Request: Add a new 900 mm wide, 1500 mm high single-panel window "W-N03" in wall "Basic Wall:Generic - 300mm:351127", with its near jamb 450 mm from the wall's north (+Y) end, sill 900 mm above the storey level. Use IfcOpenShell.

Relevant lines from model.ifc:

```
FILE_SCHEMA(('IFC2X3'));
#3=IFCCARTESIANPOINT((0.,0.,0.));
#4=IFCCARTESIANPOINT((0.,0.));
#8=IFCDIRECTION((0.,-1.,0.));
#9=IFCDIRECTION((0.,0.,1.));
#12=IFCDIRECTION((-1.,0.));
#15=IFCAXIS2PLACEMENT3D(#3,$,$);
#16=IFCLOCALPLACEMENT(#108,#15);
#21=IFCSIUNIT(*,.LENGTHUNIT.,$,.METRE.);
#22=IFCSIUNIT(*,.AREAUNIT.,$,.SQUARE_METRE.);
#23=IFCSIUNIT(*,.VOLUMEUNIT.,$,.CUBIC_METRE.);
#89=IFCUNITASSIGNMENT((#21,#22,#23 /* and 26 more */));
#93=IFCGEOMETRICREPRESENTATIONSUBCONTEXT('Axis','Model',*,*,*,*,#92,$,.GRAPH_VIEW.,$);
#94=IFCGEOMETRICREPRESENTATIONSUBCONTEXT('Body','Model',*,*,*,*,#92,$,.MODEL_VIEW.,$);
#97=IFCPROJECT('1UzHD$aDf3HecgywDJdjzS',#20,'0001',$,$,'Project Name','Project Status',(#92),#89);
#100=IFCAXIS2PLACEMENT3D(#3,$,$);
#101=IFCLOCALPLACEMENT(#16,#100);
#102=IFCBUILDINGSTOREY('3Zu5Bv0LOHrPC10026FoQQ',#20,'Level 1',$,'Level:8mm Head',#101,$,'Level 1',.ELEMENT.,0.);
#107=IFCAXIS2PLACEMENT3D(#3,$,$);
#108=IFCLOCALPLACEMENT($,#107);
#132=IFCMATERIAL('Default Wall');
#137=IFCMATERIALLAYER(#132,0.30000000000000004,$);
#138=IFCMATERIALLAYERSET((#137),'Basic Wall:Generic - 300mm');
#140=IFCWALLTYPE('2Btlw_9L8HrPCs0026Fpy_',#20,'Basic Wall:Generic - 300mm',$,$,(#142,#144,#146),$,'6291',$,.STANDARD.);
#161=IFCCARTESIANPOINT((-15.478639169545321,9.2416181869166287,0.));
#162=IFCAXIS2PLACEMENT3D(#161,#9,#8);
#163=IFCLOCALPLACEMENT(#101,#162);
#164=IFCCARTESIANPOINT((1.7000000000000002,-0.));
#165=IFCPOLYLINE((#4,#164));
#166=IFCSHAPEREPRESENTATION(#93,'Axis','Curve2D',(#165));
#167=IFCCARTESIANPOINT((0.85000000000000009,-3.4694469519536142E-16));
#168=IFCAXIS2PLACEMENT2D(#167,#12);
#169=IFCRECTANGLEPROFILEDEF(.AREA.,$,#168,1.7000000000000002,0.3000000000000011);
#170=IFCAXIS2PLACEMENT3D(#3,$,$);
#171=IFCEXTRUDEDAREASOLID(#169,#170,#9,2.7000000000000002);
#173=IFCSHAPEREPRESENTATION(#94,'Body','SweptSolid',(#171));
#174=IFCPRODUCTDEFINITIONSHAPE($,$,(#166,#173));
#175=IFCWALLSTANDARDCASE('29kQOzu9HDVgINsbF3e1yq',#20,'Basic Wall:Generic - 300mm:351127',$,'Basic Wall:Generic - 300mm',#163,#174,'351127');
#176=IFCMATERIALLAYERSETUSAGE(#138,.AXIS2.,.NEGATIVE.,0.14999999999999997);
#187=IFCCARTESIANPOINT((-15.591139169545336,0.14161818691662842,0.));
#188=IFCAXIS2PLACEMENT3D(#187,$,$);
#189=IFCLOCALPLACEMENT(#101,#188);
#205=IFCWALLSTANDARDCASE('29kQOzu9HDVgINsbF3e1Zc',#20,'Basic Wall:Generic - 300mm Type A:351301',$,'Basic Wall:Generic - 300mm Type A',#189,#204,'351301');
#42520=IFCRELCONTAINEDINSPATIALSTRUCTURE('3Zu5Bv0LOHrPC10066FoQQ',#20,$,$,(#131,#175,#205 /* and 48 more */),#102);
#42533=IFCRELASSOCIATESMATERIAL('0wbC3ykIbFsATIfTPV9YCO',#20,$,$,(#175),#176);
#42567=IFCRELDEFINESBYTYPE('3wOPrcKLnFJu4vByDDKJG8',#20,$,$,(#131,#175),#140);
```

```python
import numpy as np
import ifcopenshell
import ifcopenshell.api.feature
import ifcopenshell.api.geometry
import ifcopenshell.api.root
import ifcopenshell.api.spatial
import ifcopenshell.api.type
import ifcopenshell.geom
import ifcopenshell.util.element
import ifcopenshell.util.placement
import ifcopenshell.util.representation
import ifcopenshell.util.shape
import ifcopenshell.util.unit

model = ifcopenshell.open("model.ifc")
unit_scale = ifcopenshell.util.unit.calculate_unit_scale(model)
settings = ifcopenshell.geom.settings()


def volume(element):
    """Net volume in cubic metres, openings subtracted."""
    shape = ifcopenshell.geom.create_shape(settings, element)
    return ifcopenshell.util.shape.get_volume(shape.geometry)


wall = model.by_guid("29kQOzu9HDVgINsbF3e1yq")
storey = ifcopenshell.util.element.get_container(wall, ifc_class="IfcBuildingStorey")
context = ifcopenshell.util.representation.get_context(model, "Model", "Body", "MODEL_VIEW")
before = volume(wall)

width, height, from_end, sill = 0.9, 1.5, 0.45, 0.9  # metres

# The wall runs along its own X axis, and the end named is its -X end.
wall_shape = ifcopenshell.geom.create_shape(settings, wall)
x, y, z = ifcopenshell.util.shape.get_vertices(wall_shape.geometry).T
start = x.min() + from_end
face, thickness = float(y.min()), float(y.max() - y.min())
wall_matrix = ifcopenshell.util.placement.get_local_placement(wall.ObjectPlacement)
level = ifcopenshell.util.placement.get_local_placement(storey.ObjectPlacement)[2, 3]


def in_wall(x, y):
    """Placement at x, y metres in the wall's axes, at sill height."""
    matrix = wall_matrix.copy()
    matrix[:, 3] = wall_matrix @ np.array([x / unit_scale, y / unit_scale, 0.0, 1.0])
    matrix[2, 3] = level + sill / unit_scale
    return matrix


# Opening: a box that overshoots both wall faces by 50 mm.
opening = ifcopenshell.api.root.create_entity(model, ifc_class="IfcOpeningElement")
box = ifcopenshell.api.geometry.add_wall_representation(
    model, context=context, length=width, height=height, thickness=thickness + 0.1
)
ifcopenshell.api.geometry.assign_representation(model, product=opening, representation=box)
ifcopenshell.api.geometry.edit_object_placement(model, product=opening, matrix=in_wall(start, face - 0.05), is_si=False)
ifcopenshell.api.feature.add_feature(model, feature=opening, element=wall)

window = ifcopenshell.api.root.create_entity(model, ifc_class="IfcWindow", name="W-N03")
window.OverallWidth, window.OverallHeight = width / unit_scale, height / unit_scale
body = ifcopenshell.api.geometry.add_window_representation(
    model,
    context=context,
    overall_width=window.OverallWidth,
    overall_height=window.OverallHeight,
    partition_type="SINGLE_PANEL",
)
ifcopenshell.api.geometry.assign_representation(model, product=window, representation=body)
ifcopenshell.api.spatial.assign_container(model, products=[window], relating_structure=storey)
fills = ifcopenshell.api.feature.add_filling(model, opening=opening, element=window)
fills.OwnerHistory = window.OwnerHistory  # required in IFC2X3

# IFC2X3 keeps the operation on the window style.
style = ifcopenshell.api.root.create_entity(model, ifc_class="IfcWindowStyle", name="W-N03")
style.OperationType, style.ConstructionType = "SINGLE_PANEL", "NOTDEFINED"
style.ParameterTakesPrecedence = style.Sizeable = False
ifcopenshell.api.type.assign_type(model, related_objects=[window], relating_type=style)

# Centre the window in the wall's thickness.
ifcopenshell.api.geometry.edit_object_placement(model, product=window, matrix=in_wall(start, face), is_si=False)
window_shape = ifcopenshell.geom.create_shape(settings, window)
depth = ifcopenshell.util.shape.get_vertices(window_shape.geometry)[:, 1]
offset = face + thickness / 2 - (depth.min() + depth.max()) / 2
ifcopenshell.api.geometry.edit_object_placement(model, product=window, matrix=in_wall(start, offset), is_si=False)

after = volume(wall)

print(f"wall volume {before:.3f} -> {after:.3f} m3")

model.write("model_edited.ifc")
```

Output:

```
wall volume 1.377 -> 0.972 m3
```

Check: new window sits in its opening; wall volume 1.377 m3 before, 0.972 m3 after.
